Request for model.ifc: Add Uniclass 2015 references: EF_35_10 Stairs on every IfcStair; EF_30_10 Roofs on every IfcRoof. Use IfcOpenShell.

First a look at what the model holds.

```python
import ifcopenshell

model = ifcopenshell.open("model.ifc")
print(model.schema)
print("classifications:", [c.Name for c in model.by_type("IfcClassification")])
for ifc_class in ("IfcDoor", "IfcRoof", "IfcStair", "IfcWall", "IfcWindow"):
    print(ifc_class, len(model.by_type(ifc_class)))
```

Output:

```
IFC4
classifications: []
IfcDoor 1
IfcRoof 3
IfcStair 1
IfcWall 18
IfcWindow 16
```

```python
import ifcopenshell
import ifcopenshell.api.classification

model = ifcopenshell.open("model.ifc")

system = ifcopenshell.api.classification.add_classification(model, classification="Uniclass 2015")

codes = {
    "IfcStair": ("EF_35_10", "Stairs"),
    "IfcRoof": ("EF_30_10", "Roofs"),
}
for ifc_class, (code, name) in codes.items():
    products = model.by_type(ifc_class)
    ifcopenshell.api.classification.add_reference(
        model, products=products, classification=system, identification=code, name=name
    )
    print(code, len(products))

model.write("model_v2.ifc")
```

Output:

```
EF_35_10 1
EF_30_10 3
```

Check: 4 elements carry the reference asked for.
